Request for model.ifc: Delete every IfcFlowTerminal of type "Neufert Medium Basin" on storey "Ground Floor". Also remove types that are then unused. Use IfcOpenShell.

First a look at what the model holds.

```python
import ifcopenshell
import ifcopenshell.util.element

model = ifcopenshell.open("model.ifc")
print(model.schema)
storey = next(s for s in model.by_type("IfcBuildingStorey") if s.Name == "Ground Floor")
terminals = [e for e in ifcopenshell.util.element.get_decomposition(storey) if e.is_a("IfcFlowTerminal")]
seen = {}
for e in terminals:
    element_type = ifcopenshell.util.element.get_type(e)
    name = element_type.Name if element_type not in (None, e) else None
    seen[name] = seen.get(name, 0) + 1
for name, count in sorted(seen.items(), key=str):
    print(count, "x", name)
```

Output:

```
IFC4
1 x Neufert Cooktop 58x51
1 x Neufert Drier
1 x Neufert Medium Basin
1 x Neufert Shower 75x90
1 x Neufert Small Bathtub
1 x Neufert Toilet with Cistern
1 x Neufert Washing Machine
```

```python
import ifcopenshell
import ifcopenshell.api.root
import ifcopenshell.util.element

model = ifcopenshell.open("model.ifc")

storey = next(s for s in model.by_type("IfcBuildingStorey") if s.Name == "Ground Floor")
terminals = [e for e in ifcopenshell.util.element.get_decomposition(storey) if e.is_a("IfcFlowTerminal")]
targets = [e for e in terminals if (t := ifcopenshell.util.element.get_type(e)) not in (None, e) and t.Name == "Neufert Medium Basin"]
types = {ifcopenshell.util.element.get_type(e) for e in targets} - {None, *targets}

for e in targets:
    ifcopenshell.api.root.remove_product(model, product=e)
print(len(targets), "removed")

unused = [t for t in types if not ifcopenshell.util.element.get_types(t)]
for t in unused:
    ifcopenshell.api.root.remove_product(model, product=t)
print(len(unused), "unused types removed")

model.write("model-out.ifc")
```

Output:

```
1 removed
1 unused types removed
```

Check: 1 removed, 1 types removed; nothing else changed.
